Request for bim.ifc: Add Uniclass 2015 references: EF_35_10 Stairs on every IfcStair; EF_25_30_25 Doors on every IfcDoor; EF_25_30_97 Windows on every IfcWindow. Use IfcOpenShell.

First a look at what the model holds.

```python
import ifcopenshell

model = ifcopenshell.open("bim.ifc")
print(model.schema)
print("classifications:", [c.Name for c in model.by_type("IfcClassification")])
for ifc_class in ("IfcDoor", "IfcRoof", "IfcStair", "IfcWall", "IfcWindow"):
    print(ifc_class, len(model.by_type(ifc_class)))
```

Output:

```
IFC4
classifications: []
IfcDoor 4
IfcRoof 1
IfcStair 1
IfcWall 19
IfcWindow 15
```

```python
import ifcopenshell
import ifcopenshell.api.classification

model = ifcopenshell.open("bim.ifc")

system = ifcopenshell.api.classification.add_classification(model, classification="Uniclass 2015")

codes = {
    "IfcStair": ("EF_35_10", "Stairs"),
    "IfcDoor": ("EF_25_30_25", "Doors"),
    "IfcWindow": ("EF_25_30_97", "Windows"),
}
for ifc_class, (code, name) in codes.items():
    products = model.by_type(ifc_class)
    ifcopenshell.api.classification.add_reference(
        model, products=products, classification=system, identification=code, name=name
    )
    print(code, len(products))

model.write("bim_rev.ifc")
```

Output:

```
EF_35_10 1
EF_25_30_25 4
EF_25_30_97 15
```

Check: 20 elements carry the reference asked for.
